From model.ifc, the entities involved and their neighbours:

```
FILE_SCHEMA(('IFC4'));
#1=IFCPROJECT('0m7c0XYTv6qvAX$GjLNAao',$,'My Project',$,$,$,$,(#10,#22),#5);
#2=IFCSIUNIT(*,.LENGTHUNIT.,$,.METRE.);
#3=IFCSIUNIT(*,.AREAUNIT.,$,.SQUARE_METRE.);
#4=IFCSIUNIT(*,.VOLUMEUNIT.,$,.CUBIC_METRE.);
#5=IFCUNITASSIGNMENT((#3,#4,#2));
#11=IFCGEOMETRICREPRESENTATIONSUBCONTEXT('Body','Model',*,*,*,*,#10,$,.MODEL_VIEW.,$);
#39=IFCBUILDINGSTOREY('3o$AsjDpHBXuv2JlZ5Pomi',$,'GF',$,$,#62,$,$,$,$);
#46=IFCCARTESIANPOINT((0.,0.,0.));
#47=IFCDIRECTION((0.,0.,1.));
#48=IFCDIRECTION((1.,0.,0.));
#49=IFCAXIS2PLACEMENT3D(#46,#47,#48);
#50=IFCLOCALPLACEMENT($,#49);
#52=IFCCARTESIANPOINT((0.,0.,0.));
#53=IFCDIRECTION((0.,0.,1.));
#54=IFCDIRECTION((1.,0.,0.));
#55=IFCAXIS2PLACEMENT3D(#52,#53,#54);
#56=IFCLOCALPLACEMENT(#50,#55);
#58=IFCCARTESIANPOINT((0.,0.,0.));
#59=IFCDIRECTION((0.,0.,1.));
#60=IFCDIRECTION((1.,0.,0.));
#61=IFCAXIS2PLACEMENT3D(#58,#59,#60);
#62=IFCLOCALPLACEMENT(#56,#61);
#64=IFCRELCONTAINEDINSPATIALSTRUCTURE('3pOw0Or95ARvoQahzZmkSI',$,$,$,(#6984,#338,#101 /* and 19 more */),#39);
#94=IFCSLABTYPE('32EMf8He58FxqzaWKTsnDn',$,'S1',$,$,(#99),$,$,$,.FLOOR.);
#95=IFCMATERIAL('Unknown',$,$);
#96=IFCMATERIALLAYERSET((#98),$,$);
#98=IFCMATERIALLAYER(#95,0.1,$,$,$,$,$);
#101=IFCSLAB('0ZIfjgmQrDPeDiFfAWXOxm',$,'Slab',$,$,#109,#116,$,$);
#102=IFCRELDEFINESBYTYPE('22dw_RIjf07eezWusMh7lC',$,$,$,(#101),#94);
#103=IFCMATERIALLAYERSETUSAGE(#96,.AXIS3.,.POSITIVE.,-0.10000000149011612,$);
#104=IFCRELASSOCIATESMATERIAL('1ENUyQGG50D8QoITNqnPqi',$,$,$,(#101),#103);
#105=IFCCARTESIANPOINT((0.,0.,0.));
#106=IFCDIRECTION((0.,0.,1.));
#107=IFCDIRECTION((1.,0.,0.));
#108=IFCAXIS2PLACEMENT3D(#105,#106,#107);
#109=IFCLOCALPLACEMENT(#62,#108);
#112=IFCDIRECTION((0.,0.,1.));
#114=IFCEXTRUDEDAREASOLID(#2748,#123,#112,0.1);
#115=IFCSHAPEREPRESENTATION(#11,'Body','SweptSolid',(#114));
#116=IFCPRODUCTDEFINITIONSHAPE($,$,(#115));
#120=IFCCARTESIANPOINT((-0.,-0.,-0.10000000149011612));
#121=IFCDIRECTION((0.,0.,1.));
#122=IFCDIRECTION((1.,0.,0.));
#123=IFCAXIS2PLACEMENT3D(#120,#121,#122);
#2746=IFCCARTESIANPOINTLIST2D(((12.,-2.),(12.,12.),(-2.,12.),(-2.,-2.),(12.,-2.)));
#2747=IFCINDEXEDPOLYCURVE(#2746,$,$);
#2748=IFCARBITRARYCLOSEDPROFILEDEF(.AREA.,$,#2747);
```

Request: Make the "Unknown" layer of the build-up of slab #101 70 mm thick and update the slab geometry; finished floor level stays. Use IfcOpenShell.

```python
import ifcopenshell
import ifcopenshell.util.element
import ifcopenshell.util.representation

model = ifcopenshell.open("model.ifc")

layer_set = model.by_id(96)
layer = next(l for l in layer_set.MaterialLayers if l.Material and l.Material.Name == "Unknown")
change = 0.07 - layer.LayerThickness
layer.LayerThickness += change

# Geometry does not follow the layer set by itself.
slabs = [e for e in ifcopenshell.util.element.get_elements_by_material(model, layer_set) if e.is_a("IfcSlab")]
for slab in sorted(slabs, key=lambda e: e.id()):
    body = ifcopenshell.util.representation.get_representation(slab, "Model", "Body")
    solid = body.Items[0]
    old_depth = solid.Depth
    solid.Depth += change
    # Extruded upwards: lower the start of the extrusion so the top stays.
    x, y, z = solid.Position.Location.Coordinates
    solid.Position.Location = model.createIfcCartesianPoint((x, y, z - change))
    print(slab.id(), f"{old_depth:g} -> {solid.Depth:g}")

# The layers are counted up from the underside, which has moved.
for usage in {ifcopenshell.util.element.get_material(slab) for slab in slabs}:
    usage.OffsetFromReferenceLine -= change

model.write("model_rev.ifc")
```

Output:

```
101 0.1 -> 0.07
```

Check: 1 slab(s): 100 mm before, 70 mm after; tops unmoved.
